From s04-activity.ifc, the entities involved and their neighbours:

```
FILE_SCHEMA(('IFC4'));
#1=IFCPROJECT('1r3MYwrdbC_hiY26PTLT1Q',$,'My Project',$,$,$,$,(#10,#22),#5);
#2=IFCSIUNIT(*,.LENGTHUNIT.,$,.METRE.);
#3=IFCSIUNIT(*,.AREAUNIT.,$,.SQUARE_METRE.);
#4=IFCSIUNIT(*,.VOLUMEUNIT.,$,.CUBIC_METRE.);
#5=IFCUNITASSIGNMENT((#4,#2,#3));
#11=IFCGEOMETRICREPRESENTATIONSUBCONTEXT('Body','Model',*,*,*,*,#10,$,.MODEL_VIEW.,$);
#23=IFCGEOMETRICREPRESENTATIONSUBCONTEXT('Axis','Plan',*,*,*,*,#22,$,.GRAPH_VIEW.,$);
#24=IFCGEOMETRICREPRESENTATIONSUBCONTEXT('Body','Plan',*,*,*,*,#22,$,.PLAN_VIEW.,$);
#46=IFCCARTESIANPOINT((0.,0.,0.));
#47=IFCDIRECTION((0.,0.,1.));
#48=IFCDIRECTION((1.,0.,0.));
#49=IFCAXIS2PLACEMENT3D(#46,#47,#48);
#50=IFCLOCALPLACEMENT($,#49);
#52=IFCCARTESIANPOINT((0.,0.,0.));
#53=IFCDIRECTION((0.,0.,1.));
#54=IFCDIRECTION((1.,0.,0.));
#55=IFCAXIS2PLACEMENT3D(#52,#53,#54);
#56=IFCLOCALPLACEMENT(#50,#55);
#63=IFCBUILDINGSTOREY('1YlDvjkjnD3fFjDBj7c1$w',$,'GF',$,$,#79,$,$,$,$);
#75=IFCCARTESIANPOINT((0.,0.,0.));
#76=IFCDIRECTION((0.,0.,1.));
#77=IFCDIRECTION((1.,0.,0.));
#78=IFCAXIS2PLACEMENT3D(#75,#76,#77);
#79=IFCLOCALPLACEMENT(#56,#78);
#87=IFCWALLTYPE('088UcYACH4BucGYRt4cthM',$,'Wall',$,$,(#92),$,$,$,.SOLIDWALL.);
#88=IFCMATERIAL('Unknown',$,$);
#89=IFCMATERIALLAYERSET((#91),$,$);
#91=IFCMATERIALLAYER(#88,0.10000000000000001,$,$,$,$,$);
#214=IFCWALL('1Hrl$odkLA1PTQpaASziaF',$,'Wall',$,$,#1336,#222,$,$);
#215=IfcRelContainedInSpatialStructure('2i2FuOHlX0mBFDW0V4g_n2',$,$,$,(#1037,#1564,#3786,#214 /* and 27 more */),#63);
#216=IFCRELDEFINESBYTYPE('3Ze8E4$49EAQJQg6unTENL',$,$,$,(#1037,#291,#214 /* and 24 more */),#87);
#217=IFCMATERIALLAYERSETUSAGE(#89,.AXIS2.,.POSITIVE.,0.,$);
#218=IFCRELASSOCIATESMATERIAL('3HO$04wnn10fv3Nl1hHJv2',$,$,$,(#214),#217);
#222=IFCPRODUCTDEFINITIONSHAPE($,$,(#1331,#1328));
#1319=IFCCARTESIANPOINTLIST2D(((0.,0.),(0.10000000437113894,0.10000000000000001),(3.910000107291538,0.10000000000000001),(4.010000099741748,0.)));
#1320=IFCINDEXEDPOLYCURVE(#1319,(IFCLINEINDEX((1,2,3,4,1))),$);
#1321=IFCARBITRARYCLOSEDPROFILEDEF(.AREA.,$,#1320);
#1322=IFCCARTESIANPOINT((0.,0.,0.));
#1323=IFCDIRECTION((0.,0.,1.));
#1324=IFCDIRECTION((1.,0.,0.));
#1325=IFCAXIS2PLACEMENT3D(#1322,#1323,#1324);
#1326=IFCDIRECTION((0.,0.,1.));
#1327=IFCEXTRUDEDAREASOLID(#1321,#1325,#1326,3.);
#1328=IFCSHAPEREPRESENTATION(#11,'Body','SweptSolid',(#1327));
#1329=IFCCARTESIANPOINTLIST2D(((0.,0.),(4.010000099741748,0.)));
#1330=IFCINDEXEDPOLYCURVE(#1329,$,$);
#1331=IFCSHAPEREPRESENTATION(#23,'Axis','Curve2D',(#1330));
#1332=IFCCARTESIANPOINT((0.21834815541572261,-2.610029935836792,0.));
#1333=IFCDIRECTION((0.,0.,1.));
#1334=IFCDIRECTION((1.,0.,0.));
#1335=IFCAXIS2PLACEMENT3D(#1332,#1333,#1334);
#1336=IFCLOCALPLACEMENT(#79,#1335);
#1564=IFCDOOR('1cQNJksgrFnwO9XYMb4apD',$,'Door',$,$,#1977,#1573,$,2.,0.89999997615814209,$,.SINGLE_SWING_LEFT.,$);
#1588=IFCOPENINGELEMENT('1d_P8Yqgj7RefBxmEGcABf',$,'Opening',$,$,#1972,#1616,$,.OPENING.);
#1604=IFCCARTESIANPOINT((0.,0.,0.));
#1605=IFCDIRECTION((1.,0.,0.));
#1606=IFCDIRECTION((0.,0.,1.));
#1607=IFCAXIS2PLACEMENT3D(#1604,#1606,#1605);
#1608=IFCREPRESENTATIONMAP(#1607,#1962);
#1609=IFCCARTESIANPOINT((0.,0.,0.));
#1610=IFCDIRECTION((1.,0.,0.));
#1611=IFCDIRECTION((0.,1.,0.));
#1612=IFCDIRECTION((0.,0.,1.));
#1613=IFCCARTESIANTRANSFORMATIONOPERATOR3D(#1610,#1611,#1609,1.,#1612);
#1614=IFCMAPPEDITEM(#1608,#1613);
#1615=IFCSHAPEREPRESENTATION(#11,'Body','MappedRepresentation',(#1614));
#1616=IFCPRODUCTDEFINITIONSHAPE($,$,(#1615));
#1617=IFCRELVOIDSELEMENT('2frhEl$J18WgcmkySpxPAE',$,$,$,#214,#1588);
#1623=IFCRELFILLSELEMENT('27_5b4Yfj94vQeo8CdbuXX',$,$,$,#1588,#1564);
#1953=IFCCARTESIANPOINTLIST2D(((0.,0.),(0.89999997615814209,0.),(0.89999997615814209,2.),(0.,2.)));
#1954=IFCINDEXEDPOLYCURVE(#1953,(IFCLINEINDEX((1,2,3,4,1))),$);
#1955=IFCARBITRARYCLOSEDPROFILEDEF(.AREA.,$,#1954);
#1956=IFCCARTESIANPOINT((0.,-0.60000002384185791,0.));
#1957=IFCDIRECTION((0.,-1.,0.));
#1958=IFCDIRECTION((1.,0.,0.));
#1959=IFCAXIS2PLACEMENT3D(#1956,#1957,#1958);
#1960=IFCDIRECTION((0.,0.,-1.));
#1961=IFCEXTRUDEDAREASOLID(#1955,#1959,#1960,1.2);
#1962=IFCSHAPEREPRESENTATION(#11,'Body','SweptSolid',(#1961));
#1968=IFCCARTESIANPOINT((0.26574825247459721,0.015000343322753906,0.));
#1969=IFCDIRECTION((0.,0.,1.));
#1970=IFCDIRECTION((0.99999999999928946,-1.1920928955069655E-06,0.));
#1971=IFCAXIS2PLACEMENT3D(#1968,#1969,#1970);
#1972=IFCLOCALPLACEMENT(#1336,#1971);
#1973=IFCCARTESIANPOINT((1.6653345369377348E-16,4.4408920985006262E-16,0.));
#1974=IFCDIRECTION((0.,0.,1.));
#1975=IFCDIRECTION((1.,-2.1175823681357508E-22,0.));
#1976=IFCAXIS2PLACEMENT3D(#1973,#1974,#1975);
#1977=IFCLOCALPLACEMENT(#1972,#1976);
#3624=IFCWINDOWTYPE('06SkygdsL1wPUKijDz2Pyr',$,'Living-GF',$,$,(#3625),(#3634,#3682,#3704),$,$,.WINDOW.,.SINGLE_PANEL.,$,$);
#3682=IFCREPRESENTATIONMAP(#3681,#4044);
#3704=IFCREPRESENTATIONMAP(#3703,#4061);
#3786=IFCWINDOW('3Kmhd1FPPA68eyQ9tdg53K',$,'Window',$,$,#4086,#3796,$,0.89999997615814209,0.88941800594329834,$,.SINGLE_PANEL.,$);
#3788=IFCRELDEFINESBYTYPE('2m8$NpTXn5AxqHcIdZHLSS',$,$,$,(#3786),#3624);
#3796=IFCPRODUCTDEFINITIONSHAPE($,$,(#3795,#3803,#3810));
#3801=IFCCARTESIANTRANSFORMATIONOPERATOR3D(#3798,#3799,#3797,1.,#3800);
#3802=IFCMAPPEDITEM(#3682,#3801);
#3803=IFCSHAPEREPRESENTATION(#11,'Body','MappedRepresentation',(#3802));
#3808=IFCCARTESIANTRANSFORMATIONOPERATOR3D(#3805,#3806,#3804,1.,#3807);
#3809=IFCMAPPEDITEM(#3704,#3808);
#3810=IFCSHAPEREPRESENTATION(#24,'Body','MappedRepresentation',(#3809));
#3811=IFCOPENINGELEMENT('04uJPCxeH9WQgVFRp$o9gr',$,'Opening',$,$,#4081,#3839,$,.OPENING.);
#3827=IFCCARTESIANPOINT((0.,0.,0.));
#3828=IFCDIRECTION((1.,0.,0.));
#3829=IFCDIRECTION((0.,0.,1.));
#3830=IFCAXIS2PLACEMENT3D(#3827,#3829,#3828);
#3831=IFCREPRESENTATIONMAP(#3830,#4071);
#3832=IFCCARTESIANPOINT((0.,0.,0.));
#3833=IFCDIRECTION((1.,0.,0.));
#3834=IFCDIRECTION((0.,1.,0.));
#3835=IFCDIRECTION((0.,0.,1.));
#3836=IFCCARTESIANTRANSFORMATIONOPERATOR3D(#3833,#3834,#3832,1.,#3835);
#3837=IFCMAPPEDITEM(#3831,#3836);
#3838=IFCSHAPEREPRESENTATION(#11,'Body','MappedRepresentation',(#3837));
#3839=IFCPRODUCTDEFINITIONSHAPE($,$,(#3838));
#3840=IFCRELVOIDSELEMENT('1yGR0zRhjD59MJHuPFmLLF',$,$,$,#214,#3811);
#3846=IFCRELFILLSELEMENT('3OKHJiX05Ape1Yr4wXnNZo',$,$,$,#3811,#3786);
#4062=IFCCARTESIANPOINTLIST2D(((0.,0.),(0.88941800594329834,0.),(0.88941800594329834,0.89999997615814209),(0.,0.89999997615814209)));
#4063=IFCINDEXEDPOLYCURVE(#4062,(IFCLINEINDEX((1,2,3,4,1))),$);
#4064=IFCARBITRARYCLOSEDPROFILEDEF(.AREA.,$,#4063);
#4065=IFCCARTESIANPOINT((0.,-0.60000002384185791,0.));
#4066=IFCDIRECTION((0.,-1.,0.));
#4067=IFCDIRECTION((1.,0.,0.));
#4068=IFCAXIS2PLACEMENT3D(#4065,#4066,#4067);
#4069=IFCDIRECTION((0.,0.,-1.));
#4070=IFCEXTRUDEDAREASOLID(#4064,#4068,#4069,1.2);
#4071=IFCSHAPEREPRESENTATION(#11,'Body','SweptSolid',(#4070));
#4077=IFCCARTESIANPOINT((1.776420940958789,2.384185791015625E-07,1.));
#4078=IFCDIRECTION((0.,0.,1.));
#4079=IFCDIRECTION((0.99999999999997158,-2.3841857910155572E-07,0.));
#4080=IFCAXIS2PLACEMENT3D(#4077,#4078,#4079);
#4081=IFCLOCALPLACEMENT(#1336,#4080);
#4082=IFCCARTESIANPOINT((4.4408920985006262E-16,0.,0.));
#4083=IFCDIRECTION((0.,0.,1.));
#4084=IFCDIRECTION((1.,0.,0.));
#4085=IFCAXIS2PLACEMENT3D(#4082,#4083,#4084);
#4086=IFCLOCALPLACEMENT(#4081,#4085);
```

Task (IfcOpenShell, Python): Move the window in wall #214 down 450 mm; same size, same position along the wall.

```python
import numpy as np
import ifcopenshell
import ifcopenshell.api.geometry
import ifcopenshell.util.placement
import ifcopenshell.util.unit

model = ifcopenshell.open("s04-activity.ifc")
unit_scale = ifcopenshell.util.unit.calculate_unit_scale(model)

window = model.by_guid("3Kmhd1FPPA68eyQ9tdg53K")
opening = window.FillsVoids[0].RelatingOpeningElement
dz = -0.45 / unit_scale

shift = np.array([0.0, 0.0, dz])
# The window is placed relative to its opening, so it follows when the opening moves.
matrix = ifcopenshell.util.placement.get_local_placement(opening.ObjectPlacement)
matrix[:3, 3] += shift
ifcopenshell.api.geometry.edit_object_placement(
    model, product=opening, matrix=matrix, is_si=False, should_transform_children=True
)

print(f"moved by {dz * unit_scale:+.3f} m")

model.write("s04-activity_updated.ifc")
```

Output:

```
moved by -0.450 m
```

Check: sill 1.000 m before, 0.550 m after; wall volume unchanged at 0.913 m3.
